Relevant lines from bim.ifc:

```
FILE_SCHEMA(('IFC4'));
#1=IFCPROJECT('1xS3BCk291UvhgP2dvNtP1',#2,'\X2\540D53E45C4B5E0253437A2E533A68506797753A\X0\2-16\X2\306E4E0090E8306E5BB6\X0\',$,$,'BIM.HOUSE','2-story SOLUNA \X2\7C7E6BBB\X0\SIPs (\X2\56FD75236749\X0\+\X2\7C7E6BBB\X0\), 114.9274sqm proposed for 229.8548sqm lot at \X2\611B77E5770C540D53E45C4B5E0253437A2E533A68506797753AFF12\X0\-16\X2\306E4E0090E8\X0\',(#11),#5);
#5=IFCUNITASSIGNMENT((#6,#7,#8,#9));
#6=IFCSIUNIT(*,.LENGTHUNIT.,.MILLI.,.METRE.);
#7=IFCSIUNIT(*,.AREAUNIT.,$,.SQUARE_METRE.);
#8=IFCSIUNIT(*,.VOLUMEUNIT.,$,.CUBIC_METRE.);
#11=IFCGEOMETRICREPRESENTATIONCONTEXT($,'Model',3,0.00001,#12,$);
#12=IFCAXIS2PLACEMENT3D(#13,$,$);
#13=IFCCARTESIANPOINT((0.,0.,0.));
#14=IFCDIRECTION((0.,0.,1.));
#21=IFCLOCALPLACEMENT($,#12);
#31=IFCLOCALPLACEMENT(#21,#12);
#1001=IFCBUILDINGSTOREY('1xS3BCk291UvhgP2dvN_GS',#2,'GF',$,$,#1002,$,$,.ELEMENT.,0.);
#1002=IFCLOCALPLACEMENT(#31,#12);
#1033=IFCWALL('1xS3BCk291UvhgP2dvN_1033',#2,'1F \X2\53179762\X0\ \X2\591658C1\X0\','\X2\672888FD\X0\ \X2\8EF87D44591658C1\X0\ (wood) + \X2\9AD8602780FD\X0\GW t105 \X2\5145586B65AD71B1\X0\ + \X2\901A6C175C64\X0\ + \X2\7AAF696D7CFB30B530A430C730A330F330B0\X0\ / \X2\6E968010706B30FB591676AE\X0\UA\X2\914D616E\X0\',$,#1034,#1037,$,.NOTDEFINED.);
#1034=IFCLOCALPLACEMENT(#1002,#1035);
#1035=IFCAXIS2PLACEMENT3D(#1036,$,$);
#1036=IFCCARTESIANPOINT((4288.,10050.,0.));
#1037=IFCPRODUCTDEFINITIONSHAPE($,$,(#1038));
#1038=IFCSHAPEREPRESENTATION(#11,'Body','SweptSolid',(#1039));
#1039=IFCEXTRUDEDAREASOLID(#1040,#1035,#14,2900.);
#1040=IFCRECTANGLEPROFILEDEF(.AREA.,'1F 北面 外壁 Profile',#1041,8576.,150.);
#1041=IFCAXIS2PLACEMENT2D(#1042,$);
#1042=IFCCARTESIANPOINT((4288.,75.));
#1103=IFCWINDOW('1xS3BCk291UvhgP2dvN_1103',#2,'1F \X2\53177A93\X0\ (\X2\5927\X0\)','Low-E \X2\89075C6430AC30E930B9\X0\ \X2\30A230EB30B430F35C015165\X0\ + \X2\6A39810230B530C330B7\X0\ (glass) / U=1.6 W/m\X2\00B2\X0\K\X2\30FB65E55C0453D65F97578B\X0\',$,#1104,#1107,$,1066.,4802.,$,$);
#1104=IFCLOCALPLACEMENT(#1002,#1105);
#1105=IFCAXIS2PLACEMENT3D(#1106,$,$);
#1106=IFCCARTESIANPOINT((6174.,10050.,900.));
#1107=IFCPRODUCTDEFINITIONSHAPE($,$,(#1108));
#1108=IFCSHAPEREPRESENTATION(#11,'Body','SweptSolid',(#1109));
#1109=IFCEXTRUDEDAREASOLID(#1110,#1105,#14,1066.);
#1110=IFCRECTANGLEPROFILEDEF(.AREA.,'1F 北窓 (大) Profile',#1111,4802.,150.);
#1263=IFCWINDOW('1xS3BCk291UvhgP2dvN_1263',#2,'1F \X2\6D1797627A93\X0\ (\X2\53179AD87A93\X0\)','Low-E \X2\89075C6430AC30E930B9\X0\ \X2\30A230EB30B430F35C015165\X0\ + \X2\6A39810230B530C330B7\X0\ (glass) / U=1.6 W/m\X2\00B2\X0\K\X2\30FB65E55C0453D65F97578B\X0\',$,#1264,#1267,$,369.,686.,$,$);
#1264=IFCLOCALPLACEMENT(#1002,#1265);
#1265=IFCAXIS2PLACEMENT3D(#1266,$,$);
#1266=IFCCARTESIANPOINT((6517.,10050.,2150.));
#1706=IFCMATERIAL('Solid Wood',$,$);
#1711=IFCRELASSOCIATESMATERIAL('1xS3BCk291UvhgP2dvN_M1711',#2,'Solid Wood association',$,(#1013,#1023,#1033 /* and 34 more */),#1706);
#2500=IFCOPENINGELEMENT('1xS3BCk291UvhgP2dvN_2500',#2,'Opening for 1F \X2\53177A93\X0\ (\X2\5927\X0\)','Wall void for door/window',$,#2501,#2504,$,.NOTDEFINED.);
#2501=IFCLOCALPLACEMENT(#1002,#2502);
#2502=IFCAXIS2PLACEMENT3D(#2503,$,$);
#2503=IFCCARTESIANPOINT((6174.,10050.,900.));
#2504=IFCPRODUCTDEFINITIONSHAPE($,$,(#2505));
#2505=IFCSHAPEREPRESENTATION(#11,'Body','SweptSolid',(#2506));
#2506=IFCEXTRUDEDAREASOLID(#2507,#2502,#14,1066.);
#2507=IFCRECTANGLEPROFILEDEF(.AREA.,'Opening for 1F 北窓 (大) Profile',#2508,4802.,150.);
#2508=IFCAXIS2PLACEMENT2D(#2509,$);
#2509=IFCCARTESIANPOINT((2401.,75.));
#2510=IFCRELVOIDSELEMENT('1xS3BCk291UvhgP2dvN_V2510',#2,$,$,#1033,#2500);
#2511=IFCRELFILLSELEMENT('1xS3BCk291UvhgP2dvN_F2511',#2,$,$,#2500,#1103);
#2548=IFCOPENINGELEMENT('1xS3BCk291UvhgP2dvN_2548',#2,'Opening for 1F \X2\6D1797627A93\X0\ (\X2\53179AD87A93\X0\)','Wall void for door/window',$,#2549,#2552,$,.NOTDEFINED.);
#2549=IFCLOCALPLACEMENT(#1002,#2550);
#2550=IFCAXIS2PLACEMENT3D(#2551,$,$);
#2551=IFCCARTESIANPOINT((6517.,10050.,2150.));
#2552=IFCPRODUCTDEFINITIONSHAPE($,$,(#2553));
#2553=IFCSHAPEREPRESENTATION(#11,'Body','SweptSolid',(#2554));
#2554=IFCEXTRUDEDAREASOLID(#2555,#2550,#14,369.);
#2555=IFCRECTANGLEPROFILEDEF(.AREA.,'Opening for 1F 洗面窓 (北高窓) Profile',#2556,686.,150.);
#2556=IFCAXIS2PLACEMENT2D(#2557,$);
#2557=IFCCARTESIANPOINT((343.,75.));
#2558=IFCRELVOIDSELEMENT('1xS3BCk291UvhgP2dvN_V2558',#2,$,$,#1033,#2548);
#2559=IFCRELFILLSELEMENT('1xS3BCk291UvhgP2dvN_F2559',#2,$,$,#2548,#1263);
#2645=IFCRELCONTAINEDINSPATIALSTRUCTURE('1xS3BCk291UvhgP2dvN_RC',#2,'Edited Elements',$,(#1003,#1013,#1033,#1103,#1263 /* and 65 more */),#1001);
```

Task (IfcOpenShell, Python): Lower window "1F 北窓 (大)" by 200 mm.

```python
import numpy as np
import ifcopenshell
import ifcopenshell.api.geometry
import ifcopenshell.util.placement
import ifcopenshell.util.unit

model = ifcopenshell.open("bim.ifc")
unit_scale = ifcopenshell.util.unit.calculate_unit_scale(model)

window = model.by_id(1103)
opening = window.FillsVoids[0].RelatingOpeningElement
dz = -0.2 / unit_scale

shift = np.array([0.0, 0.0, dz])
# The window is not placed relative to its opening, so move both.
for product in (opening, window):
    matrix = ifcopenshell.util.placement.get_local_placement(product.ObjectPlacement)
    matrix[:3, 3] += shift
    ifcopenshell.api.geometry.edit_object_placement(model, product=product, matrix=matrix, is_si=False)

print(f"moved by {dz * unit_scale:+.3f} m")

model.write("bim_updated.ifc")
```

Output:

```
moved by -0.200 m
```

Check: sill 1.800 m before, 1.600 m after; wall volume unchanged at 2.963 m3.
